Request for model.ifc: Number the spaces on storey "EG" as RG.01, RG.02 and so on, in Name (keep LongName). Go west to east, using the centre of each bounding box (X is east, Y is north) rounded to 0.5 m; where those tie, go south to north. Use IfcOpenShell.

First a look at what the model holds.

```python
import ifcopenshell
import ifcopenshell.util.element
import ifcopenshell.util.placement

model = ifcopenshell.open("model.ifc")
print(model.schema)
storey = next(s for s in model.by_type("IfcBuildingStorey") if s.Name == "EG")
spaces = [e for e in ifcopenshell.util.element.get_decomposition(storey) if e.is_a("IfcSpace")]
for e in sorted(spaces, key=lambda e: e.id()):
    origin = ifcopenshell.util.placement.get_local_placement(e.ObjectPlacement)[:3, 3]
    print(e.id(), e.Name, e.LongName, origin.round(2) + 0.0, sep=" | ")
```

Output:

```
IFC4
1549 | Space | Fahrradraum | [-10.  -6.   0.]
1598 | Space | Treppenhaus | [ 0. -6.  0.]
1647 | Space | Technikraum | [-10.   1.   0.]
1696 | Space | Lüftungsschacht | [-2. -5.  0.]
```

```python
import ifcopenshell
import ifcopenshell.geom
import ifcopenshell.util.element
import ifcopenshell.util.shape

model = ifcopenshell.open("model.ifc")
settings = ifcopenshell.geom.settings()
settings.set("use-world-coords", True)


def centre(element):
    shape = ifcopenshell.geom.create_shape(settings, element)
    return ifcopenshell.util.shape.get_bbox_centroid(shape.geometry)


storey = next(s for s in model.by_type("IfcBuildingStorey") if s.Name == "EG")
spaces = [e for e in ifcopenshell.util.element.get_decomposition(storey) if e.is_a("IfcSpace")]

# Insertion points can sit at a corner or the storey origin, so sort by the geometry (in metres).
centres = {e: centre(e) for e in spaces}
spaces.sort(key=lambda e: (round(centres[e][0] / 0.5), centres[e][1]))

for i, e in enumerate(spaces, start=1):
    number = f"RG.{i:02d}"
    e.Name = number
    print(e.id(), number)

model.write("model_updated.ifc")
```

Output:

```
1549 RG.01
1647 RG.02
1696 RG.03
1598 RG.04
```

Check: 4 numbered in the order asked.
